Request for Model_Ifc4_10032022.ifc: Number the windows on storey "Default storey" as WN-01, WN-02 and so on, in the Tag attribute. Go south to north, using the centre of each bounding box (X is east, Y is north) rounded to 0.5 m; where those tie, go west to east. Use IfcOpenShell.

First a look at what the model holds.

```python
import ifcopenshell
import ifcopenshell.util.element
import ifcopenshell.util.placement

model = ifcopenshell.open("Model_Ifc4_10032022.ifc")
print(model.schema)
storey = next(s for s in model.by_type("IfcBuildingStorey") if s.Name == "Default storey")
windows = [e for e in ifcopenshell.util.element.get_decomposition(storey) if e.is_a("IfcWindow")]
for e in sorted(windows, key=lambda e: e.id()):
    origin = ifcopenshell.util.placement.get_local_placement(e.ObjectPlacement)[:3, 3]
    print(e.id(), e.Tag, e.Name, origin.round(2) + 0.0, sep=" | ")
```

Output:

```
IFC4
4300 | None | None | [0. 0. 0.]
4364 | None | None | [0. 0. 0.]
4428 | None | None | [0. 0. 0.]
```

```python
import ifcopenshell
import ifcopenshell.geom
import ifcopenshell.util.element
import ifcopenshell.util.shape

model = ifcopenshell.open("Model_Ifc4_10032022.ifc")
settings = ifcopenshell.geom.settings()
settings.set("use-world-coords", True)


def centre(element):
    shape = ifcopenshell.geom.create_shape(settings, element)
    return ifcopenshell.util.shape.get_bbox_centroid(shape.geometry)


storey = next(s for s in model.by_type("IfcBuildingStorey") if s.Name == "Default storey")
windows = [e for e in ifcopenshell.util.element.get_decomposition(storey) if e.is_a("IfcWindow")]

# Insertion points can sit at a corner or the storey origin, so sort by the geometry (in metres).
centres = {e: centre(e) for e in windows}
windows.sort(key=lambda e: (round(centres[e][1] / 0.5), centres[e][0]))

for i, e in enumerate(windows, start=1):
    number = f"WN-{i:02d}"
    e.Tag = number
    print(e.id(), number)

model.write("Model_Ifc4_10032022_updated.ifc")
```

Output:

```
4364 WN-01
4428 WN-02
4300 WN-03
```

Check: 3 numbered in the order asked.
